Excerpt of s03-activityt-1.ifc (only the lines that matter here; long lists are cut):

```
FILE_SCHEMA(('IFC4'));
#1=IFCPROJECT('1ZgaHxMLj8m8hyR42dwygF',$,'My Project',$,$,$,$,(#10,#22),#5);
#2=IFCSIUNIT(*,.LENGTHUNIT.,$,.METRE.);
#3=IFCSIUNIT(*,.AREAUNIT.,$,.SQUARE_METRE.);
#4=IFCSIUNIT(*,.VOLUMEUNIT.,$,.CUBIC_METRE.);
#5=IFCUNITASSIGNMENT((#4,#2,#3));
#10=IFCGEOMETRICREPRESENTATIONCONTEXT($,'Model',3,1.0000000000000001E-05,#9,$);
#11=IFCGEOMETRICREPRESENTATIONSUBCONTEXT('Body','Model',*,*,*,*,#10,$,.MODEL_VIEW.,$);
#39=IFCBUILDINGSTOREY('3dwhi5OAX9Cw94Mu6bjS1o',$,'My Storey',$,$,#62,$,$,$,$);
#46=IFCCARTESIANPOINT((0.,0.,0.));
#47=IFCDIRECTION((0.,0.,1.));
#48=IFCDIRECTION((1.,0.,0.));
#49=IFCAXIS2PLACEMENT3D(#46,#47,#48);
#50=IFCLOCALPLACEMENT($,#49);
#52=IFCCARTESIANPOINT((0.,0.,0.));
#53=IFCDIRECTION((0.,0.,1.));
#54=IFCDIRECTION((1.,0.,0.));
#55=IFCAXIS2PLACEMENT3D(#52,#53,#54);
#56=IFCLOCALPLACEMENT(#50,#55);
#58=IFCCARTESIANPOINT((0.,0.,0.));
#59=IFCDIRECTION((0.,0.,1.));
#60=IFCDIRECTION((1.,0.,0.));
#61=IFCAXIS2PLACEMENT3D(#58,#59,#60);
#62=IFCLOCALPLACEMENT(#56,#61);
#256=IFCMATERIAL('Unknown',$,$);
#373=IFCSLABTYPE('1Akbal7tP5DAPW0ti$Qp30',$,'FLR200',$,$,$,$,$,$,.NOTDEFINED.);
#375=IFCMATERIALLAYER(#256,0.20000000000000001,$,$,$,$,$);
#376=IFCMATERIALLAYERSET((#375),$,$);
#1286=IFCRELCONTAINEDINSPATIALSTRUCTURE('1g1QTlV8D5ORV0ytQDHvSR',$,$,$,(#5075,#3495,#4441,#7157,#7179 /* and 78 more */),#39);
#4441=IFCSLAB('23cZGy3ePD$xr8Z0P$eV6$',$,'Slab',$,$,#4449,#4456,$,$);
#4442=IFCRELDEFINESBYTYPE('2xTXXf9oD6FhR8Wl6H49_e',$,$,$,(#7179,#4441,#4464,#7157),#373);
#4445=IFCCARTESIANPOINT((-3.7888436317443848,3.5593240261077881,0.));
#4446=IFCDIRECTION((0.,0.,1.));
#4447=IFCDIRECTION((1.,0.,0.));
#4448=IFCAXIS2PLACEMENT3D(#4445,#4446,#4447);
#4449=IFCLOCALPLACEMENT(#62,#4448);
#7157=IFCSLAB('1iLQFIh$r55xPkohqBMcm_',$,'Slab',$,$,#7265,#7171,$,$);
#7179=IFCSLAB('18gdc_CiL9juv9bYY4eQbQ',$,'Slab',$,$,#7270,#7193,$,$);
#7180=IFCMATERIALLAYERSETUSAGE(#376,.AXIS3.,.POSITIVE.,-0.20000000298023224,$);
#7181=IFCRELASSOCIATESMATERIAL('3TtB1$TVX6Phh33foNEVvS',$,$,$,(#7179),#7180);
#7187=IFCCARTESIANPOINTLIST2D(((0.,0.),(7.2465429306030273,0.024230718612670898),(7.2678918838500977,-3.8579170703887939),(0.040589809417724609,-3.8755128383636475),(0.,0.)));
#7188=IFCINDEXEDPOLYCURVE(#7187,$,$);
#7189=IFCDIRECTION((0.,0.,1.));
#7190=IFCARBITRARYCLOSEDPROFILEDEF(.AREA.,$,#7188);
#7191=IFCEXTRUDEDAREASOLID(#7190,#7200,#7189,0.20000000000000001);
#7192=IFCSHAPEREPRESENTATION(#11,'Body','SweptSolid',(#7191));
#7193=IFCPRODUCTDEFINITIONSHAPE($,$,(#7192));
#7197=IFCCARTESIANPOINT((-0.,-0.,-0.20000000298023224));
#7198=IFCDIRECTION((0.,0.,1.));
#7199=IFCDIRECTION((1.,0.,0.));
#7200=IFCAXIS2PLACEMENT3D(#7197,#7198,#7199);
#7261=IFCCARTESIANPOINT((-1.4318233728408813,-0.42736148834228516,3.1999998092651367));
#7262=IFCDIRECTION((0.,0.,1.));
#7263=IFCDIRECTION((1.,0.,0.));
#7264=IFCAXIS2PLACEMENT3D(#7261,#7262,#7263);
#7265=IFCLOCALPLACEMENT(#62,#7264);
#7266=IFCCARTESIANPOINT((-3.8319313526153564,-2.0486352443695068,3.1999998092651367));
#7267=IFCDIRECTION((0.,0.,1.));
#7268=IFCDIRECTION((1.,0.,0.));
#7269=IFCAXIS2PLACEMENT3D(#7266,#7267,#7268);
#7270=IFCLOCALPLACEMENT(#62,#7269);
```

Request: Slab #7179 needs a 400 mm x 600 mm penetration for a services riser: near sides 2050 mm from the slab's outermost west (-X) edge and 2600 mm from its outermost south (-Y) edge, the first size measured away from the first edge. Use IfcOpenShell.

```python
import numpy as np
import ifcopenshell
import ifcopenshell.api.feature
import ifcopenshell.api.geometry
import ifcopenshell.api.root
import ifcopenshell.geom
import ifcopenshell.util.placement
import ifcopenshell.util.representation
import ifcopenshell.util.shape
import ifcopenshell.util.unit

model = ifcopenshell.open("s03-activityt-1.ifc")
unit_scale = ifcopenshell.util.unit.calculate_unit_scale(model)
settings = ifcopenshell.geom.settings()


def volume(element):
    """Net volume in cubic metres, openings subtracted."""
    shape = ifcopenshell.geom.create_shape(settings, element)
    return ifcopenshell.util.shape.get_volume(shape.geometry)


slab = model.by_guid("18gdc_CiL9juv9bYY4eQbQ")
before = volume(slab)

# Extent in the slab's own axes, in metres. The edges named are its -X and -Y sides.
slab_shape = ifcopenshell.geom.create_shape(settings, slab)
vertices = ifcopenshell.util.shape.get_vertices(slab_shape.geometry)
x_min, y_min, bottom = vertices.min(axis=0)
top = vertices[:, 2].max()

opening = ifcopenshell.api.root.create_entity(model, ifc_class="IfcOpeningElement", name="Services riser opening", predefined_type="OPENING")
context = ifcopenshell.util.representation.get_context(model, "Model", "Body", "MODEL_VIEW")
width, depth = 0.4, 0.6
outline = [(0.0, 0.0), (width, 0.0), (width, depth), (0.0, depth), (0.0, 0.0)]
# Overshoot both faces by 50 mm so the cut is clean.
shape = ifcopenshell.api.geometry.add_slab_representation(
    model, context=context, depth=top - bottom + 0.1, polyline=outline
)
ifcopenshell.api.geometry.assign_representation(model, product=opening, representation=shape)

matrix = ifcopenshell.util.placement.get_local_placement(slab.ObjectPlacement)
matrix[:, 3] = matrix @ np.append(np.array([x_min + 2.05, y_min + 2.6, bottom - 0.05]) / unit_scale, 1.0)
ifcopenshell.api.geometry.edit_object_placement(model, product=opening, matrix=matrix, is_si=False)
ifcopenshell.api.feature.add_feature(model, feature=opening, element=slab)

after = volume(slab)

print(f"slab volume {before:.3f} -> {after:.3f} m3")

model.write("s03-activityt-1-out.ifc")
```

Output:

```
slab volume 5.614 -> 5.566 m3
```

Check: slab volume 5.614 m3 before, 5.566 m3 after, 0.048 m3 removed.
